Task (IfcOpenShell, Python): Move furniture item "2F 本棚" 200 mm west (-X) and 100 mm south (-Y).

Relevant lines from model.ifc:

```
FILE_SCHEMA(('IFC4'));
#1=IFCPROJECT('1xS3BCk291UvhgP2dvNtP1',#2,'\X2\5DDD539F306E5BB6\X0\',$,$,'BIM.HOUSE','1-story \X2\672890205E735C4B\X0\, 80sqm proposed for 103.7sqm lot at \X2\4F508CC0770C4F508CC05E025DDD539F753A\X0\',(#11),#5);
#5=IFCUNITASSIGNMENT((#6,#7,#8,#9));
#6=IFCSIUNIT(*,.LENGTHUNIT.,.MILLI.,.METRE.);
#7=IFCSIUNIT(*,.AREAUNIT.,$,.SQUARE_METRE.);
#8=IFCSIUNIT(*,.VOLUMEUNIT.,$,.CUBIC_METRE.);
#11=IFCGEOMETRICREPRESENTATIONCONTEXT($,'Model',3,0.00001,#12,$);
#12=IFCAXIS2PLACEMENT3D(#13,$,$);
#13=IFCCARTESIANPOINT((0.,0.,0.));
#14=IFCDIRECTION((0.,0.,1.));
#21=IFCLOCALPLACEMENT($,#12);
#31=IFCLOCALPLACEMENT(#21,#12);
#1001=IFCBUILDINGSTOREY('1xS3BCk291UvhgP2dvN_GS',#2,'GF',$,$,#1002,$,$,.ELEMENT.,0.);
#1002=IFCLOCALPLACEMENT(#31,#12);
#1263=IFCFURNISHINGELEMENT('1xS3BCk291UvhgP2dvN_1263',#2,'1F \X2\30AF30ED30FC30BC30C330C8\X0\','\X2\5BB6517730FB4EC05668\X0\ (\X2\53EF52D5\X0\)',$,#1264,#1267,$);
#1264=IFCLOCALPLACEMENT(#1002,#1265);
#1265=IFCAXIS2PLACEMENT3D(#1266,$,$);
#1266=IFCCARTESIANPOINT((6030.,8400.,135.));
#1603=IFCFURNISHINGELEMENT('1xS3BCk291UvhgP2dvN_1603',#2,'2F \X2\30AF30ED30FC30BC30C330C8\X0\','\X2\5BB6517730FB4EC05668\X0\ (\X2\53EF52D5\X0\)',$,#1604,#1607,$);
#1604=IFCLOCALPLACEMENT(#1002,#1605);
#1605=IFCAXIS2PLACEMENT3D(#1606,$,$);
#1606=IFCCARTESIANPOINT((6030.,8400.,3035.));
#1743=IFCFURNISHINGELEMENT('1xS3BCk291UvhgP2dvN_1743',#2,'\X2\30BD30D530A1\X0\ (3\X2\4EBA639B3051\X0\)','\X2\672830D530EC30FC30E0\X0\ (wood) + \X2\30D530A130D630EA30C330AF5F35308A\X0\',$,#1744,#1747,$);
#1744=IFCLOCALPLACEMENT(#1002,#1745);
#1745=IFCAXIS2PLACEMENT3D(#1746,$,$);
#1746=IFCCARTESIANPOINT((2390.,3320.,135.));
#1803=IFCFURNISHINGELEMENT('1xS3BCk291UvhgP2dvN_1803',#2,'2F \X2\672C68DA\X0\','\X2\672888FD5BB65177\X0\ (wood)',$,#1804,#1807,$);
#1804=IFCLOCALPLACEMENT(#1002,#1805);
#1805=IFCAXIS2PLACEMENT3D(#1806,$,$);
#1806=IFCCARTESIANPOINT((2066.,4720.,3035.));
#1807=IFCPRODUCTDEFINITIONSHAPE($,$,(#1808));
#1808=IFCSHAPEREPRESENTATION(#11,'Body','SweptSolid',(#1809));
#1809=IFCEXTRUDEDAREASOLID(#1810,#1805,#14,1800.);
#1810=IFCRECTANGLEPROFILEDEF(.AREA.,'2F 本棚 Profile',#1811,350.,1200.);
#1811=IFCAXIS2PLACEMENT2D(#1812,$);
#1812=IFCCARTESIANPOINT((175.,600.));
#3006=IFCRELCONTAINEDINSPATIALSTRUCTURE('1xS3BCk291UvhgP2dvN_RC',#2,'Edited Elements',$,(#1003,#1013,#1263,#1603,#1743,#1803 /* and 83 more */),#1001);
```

```python
import ifcopenshell
import ifcopenshell.api.geometry
import ifcopenshell.util.placement

model = ifcopenshell.open("model.ifc")

item = model.by_guid("1xS3BCk291UvhgP2dvN_1803")
matrix = ifcopenshell.util.placement.get_local_placement(item.ObjectPlacement)
matrix[0, 3] -= 200.0
matrix[1, 3] -= 100.0
ifcopenshell.api.geometry.edit_object_placement(model, product=item, matrix=matrix, is_si=False)

print(ifcopenshell.util.placement.get_local_placement(item.ObjectPlacement).round(3) + 0.0)

model.write("model_rev.ifc")
```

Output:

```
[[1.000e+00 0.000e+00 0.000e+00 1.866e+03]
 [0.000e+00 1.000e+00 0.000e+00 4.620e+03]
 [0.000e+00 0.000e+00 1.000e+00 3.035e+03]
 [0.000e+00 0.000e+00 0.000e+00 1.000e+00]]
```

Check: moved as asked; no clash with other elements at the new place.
